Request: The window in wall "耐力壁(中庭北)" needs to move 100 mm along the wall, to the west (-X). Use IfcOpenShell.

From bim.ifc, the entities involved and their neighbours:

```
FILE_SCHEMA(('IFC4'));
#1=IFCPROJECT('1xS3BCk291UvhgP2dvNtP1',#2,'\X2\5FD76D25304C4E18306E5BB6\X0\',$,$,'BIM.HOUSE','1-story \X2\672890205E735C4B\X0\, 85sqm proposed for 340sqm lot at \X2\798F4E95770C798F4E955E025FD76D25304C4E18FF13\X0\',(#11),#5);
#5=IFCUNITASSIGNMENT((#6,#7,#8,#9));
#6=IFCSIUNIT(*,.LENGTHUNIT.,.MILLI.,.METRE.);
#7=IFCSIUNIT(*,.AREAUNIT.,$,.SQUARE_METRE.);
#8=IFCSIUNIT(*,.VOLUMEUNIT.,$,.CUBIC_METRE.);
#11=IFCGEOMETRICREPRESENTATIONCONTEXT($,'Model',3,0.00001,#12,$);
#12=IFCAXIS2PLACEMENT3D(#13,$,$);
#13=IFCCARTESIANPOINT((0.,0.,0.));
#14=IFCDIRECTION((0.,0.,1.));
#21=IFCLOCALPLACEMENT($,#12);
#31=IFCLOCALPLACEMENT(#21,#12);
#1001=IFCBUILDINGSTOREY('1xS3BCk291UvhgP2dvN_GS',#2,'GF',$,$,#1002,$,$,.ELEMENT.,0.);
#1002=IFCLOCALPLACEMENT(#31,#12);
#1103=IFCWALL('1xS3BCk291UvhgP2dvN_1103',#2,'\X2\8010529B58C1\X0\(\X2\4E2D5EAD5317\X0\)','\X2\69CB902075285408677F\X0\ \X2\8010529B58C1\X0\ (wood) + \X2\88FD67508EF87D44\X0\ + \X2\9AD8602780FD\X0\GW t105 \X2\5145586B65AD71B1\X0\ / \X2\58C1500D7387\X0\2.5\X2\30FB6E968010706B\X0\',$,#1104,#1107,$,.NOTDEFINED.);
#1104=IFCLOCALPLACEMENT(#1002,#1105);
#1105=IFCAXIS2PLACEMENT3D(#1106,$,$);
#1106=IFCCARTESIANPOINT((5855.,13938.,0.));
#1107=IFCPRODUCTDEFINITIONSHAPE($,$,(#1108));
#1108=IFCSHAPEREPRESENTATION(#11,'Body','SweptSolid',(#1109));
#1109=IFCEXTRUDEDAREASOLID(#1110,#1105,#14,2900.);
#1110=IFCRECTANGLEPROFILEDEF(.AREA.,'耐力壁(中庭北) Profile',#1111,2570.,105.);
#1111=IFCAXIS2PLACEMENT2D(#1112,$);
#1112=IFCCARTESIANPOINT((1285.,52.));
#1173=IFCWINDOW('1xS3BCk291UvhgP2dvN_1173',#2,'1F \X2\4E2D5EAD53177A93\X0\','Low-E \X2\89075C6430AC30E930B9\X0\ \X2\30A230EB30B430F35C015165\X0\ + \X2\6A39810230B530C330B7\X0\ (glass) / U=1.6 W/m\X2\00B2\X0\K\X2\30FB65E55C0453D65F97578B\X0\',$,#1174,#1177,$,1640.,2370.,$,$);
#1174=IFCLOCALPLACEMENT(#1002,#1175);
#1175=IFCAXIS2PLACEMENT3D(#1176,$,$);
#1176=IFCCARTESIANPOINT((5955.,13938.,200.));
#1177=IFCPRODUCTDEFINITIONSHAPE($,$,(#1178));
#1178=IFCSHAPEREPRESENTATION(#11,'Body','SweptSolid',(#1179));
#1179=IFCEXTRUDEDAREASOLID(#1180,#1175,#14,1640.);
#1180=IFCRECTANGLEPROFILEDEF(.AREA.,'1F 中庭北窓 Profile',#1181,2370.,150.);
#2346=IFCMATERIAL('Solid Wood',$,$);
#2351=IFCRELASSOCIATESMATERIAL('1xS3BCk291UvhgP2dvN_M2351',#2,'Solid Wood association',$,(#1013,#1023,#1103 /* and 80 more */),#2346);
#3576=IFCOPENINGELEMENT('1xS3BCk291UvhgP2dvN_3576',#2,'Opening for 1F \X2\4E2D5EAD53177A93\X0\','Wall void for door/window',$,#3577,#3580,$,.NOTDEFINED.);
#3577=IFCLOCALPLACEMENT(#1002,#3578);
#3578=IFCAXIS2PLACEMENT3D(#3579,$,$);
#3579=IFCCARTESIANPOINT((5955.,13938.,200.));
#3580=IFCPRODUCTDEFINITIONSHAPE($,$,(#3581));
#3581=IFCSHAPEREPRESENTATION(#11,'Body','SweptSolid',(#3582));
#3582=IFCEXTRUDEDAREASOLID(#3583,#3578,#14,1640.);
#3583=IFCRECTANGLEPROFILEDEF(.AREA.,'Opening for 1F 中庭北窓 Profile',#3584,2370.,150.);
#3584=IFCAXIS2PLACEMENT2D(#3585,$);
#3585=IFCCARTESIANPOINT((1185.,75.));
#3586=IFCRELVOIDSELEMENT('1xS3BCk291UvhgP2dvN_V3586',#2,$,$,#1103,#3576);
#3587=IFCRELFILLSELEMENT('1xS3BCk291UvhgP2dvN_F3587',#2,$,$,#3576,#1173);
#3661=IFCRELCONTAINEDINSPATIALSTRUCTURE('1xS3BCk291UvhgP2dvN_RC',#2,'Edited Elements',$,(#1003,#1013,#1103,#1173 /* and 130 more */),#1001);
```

```python
import ifcopenshell
import ifcopenshell.api.geometry
import ifcopenshell.util.placement
import ifcopenshell.util.unit

model = ifcopenshell.open("bim.ifc")
unit_scale = ifcopenshell.util.unit.calculate_unit_scale(model)

window = model.by_guid("1xS3BCk291UvhgP2dvN_1173")
opening = window.FillsVoids[0].RelatingOpeningElement
wall = opening.VoidsElements[0].RelatingBuildingElement

wall_matrix = ifcopenshell.util.placement.get_local_placement(wall.ObjectPlacement)
shift = wall_matrix[:3, 0] * -0.1 / unit_scale
before = ifcopenshell.util.placement.get_local_placement(window.ObjectPlacement)[:3, 3].copy()

# The window is not placed relative to its opening, so move both.
for product in (opening, window):
    matrix = ifcopenshell.util.placement.get_local_placement(product.ObjectPlacement)
    matrix[:3, 3] += shift
    ifcopenshell.api.geometry.edit_object_placement(model, product=product, matrix=matrix, is_si=False)

after = ifcopenshell.util.placement.get_local_placement(window.ObjectPlacement)[:3, 3]
print("window moved by", (after - before).round(3) + 0.0)

model.write("bim_updated.ifc")
```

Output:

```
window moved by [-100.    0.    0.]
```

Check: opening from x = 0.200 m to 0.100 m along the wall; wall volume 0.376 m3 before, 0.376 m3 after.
